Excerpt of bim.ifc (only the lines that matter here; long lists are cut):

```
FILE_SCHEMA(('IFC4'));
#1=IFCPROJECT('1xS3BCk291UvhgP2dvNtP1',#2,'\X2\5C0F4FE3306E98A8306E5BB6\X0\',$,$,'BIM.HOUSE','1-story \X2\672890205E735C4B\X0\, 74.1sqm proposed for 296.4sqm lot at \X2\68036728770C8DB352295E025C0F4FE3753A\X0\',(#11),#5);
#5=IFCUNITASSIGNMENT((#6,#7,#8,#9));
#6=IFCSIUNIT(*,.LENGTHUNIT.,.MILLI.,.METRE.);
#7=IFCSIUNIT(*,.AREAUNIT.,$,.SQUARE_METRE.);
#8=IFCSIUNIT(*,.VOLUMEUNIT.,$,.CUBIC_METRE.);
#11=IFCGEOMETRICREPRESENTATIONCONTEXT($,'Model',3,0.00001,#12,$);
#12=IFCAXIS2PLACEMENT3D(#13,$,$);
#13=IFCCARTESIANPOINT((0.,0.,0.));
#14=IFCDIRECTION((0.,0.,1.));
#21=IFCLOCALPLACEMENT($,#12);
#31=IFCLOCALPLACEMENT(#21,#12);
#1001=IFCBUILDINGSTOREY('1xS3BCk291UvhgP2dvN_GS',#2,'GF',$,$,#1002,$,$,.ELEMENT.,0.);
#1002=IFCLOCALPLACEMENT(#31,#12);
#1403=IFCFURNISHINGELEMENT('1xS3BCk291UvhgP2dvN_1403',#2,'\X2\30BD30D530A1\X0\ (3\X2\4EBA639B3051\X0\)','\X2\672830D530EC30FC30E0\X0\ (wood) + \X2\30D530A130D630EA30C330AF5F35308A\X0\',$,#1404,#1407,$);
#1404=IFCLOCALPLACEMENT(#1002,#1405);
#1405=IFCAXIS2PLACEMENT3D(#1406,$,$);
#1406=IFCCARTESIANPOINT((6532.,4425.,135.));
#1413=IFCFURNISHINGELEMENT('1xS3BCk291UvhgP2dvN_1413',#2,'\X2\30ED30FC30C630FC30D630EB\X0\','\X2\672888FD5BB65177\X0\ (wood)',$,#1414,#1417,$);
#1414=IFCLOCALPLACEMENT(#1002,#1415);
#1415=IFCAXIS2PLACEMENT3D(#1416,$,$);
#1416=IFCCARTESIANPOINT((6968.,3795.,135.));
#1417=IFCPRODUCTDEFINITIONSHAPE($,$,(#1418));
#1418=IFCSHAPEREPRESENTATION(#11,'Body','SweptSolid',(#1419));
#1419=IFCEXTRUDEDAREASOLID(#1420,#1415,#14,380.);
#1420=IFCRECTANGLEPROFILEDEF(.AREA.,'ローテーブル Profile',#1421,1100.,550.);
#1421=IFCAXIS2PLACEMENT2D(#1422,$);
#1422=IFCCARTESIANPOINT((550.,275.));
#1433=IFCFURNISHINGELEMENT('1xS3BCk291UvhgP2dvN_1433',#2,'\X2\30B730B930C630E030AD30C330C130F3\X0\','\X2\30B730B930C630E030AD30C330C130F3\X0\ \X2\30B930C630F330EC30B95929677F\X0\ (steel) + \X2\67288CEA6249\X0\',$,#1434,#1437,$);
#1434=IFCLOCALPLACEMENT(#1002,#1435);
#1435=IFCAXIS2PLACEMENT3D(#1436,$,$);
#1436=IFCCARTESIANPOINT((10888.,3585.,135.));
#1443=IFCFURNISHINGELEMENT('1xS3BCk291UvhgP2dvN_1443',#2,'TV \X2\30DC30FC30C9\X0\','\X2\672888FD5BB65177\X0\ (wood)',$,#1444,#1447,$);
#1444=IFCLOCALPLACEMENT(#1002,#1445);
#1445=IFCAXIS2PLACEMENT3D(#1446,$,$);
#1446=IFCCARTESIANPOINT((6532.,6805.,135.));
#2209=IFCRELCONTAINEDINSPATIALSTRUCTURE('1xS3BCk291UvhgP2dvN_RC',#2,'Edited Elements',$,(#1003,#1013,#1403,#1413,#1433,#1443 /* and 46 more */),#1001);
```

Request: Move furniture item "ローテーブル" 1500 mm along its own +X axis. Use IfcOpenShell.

```python
import ifcopenshell
import ifcopenshell.api.geometry
import ifcopenshell.util.placement

model = ifcopenshell.open("bim.ifc")

item = model.by_id(1413)
matrix = ifcopenshell.util.placement.get_local_placement(item.ObjectPlacement)
matrix[:3, 3] += matrix[:3, 0] * 1500.0
ifcopenshell.api.geometry.edit_object_placement(model, product=item, matrix=matrix, is_si=False)

print(ifcopenshell.util.placement.get_local_placement(item.ObjectPlacement).round(3) + 0.0)

model.write("bim-out.ifc")
```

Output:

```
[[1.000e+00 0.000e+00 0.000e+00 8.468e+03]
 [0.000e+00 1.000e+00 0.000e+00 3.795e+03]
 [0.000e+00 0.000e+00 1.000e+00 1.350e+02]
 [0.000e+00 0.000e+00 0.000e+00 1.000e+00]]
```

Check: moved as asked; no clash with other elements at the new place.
